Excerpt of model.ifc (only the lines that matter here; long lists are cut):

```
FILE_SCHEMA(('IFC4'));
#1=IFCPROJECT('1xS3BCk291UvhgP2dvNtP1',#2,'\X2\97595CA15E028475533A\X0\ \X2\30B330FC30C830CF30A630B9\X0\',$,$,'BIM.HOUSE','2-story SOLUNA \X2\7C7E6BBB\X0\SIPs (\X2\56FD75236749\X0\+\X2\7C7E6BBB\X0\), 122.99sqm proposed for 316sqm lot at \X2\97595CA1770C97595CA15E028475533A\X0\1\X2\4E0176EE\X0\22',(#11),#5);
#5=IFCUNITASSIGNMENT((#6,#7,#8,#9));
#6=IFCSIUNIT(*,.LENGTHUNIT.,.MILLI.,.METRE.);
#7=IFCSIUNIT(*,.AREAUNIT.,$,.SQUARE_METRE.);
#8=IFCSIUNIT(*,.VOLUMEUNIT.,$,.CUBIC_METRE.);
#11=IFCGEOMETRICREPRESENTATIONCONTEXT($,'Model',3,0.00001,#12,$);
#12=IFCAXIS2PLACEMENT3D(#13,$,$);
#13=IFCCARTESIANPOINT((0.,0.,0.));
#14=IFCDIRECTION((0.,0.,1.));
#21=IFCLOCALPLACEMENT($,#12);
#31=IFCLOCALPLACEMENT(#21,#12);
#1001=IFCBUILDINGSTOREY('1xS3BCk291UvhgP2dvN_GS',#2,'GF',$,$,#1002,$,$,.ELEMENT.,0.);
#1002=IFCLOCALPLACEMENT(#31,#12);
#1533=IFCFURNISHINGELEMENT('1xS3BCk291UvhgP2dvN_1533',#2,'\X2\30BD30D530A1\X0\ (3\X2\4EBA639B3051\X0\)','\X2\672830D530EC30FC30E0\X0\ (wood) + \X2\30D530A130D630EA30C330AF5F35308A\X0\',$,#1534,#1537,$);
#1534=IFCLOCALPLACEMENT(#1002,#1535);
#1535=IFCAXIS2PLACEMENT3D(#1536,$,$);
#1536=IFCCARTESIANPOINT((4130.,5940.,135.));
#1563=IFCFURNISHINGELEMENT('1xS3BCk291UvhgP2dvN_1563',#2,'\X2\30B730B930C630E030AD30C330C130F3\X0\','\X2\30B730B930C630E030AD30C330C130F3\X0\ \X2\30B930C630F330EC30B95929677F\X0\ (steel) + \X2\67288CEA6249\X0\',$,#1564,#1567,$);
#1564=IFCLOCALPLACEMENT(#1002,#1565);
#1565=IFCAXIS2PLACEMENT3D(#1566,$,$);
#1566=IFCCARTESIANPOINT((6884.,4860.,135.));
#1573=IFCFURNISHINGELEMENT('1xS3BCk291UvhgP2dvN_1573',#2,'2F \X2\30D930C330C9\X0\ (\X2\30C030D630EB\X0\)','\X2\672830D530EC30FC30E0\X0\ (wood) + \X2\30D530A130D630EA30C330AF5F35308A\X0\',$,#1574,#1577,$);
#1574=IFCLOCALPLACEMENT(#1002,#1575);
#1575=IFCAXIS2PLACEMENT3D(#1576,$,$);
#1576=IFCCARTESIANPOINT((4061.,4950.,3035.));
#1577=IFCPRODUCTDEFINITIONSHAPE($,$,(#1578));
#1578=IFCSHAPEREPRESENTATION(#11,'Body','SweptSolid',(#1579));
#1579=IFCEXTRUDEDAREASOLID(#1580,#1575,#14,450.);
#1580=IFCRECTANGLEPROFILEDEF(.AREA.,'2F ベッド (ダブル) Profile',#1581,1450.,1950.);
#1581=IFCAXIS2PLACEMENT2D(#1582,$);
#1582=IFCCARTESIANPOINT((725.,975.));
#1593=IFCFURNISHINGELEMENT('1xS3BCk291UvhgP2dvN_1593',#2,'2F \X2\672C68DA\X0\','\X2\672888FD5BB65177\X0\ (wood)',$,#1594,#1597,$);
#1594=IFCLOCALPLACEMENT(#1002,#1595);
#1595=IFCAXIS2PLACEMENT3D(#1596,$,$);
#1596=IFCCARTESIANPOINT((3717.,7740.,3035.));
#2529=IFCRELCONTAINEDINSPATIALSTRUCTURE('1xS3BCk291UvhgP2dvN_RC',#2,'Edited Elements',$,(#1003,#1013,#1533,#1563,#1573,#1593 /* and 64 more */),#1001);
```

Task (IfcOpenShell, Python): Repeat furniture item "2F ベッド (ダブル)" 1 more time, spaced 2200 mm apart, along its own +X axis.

```python
import ifcopenshell
import ifcopenshell.api.geometry
import ifcopenshell.api.root
import ifcopenshell.util.element
import ifcopenshell.util.placement
import ifcopenshell.util.unit

model = ifcopenshell.open("model.ifc")
unit_scale = ifcopenshell.util.unit.calculate_unit_scale(model)


def reuse_history(source, copy):
    """copy_class also copies each property set's owner history, people and application; keep the originals."""
    for rel in copy.IsDefinedBy:
        if rel.is_a("IfcRelDefinesByProperties") and (history := rel.RelatingPropertyDefinition.OwnerHistory):
            rel.RelatingPropertyDefinition.OwnerHistory = source.OwnerHistory
            ifcopenshell.util.element.remove_deep2(model, history)


source = model.by_guid("1xS3BCk291UvhgP2dvN_1573")
base = ifcopenshell.util.placement.get_local_placement(source.ObjectPlacement)
step = base[:3, 0] * 2.2 / unit_scale

for i in range(1, 2):
    copy = ifcopenshell.api.root.copy_class(model, product=source)
    copy.Representation = ifcopenshell.util.element.copy_deep(
        model, source.Representation, exclude=["IfcGeometricRepresentationContext", "IfcRepresentationMap"]
    )
    reuse_history(source, copy)
    matrix = base.copy()
    matrix[:3, 3] += i * step
    print("added at", matrix[:3, 3].round(3) + 0.0)
    ifcopenshell.api.geometry.edit_object_placement(model, product=copy, matrix=matrix, is_si=False)

model.write("model-out.ifc")
```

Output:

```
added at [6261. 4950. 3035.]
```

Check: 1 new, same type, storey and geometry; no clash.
